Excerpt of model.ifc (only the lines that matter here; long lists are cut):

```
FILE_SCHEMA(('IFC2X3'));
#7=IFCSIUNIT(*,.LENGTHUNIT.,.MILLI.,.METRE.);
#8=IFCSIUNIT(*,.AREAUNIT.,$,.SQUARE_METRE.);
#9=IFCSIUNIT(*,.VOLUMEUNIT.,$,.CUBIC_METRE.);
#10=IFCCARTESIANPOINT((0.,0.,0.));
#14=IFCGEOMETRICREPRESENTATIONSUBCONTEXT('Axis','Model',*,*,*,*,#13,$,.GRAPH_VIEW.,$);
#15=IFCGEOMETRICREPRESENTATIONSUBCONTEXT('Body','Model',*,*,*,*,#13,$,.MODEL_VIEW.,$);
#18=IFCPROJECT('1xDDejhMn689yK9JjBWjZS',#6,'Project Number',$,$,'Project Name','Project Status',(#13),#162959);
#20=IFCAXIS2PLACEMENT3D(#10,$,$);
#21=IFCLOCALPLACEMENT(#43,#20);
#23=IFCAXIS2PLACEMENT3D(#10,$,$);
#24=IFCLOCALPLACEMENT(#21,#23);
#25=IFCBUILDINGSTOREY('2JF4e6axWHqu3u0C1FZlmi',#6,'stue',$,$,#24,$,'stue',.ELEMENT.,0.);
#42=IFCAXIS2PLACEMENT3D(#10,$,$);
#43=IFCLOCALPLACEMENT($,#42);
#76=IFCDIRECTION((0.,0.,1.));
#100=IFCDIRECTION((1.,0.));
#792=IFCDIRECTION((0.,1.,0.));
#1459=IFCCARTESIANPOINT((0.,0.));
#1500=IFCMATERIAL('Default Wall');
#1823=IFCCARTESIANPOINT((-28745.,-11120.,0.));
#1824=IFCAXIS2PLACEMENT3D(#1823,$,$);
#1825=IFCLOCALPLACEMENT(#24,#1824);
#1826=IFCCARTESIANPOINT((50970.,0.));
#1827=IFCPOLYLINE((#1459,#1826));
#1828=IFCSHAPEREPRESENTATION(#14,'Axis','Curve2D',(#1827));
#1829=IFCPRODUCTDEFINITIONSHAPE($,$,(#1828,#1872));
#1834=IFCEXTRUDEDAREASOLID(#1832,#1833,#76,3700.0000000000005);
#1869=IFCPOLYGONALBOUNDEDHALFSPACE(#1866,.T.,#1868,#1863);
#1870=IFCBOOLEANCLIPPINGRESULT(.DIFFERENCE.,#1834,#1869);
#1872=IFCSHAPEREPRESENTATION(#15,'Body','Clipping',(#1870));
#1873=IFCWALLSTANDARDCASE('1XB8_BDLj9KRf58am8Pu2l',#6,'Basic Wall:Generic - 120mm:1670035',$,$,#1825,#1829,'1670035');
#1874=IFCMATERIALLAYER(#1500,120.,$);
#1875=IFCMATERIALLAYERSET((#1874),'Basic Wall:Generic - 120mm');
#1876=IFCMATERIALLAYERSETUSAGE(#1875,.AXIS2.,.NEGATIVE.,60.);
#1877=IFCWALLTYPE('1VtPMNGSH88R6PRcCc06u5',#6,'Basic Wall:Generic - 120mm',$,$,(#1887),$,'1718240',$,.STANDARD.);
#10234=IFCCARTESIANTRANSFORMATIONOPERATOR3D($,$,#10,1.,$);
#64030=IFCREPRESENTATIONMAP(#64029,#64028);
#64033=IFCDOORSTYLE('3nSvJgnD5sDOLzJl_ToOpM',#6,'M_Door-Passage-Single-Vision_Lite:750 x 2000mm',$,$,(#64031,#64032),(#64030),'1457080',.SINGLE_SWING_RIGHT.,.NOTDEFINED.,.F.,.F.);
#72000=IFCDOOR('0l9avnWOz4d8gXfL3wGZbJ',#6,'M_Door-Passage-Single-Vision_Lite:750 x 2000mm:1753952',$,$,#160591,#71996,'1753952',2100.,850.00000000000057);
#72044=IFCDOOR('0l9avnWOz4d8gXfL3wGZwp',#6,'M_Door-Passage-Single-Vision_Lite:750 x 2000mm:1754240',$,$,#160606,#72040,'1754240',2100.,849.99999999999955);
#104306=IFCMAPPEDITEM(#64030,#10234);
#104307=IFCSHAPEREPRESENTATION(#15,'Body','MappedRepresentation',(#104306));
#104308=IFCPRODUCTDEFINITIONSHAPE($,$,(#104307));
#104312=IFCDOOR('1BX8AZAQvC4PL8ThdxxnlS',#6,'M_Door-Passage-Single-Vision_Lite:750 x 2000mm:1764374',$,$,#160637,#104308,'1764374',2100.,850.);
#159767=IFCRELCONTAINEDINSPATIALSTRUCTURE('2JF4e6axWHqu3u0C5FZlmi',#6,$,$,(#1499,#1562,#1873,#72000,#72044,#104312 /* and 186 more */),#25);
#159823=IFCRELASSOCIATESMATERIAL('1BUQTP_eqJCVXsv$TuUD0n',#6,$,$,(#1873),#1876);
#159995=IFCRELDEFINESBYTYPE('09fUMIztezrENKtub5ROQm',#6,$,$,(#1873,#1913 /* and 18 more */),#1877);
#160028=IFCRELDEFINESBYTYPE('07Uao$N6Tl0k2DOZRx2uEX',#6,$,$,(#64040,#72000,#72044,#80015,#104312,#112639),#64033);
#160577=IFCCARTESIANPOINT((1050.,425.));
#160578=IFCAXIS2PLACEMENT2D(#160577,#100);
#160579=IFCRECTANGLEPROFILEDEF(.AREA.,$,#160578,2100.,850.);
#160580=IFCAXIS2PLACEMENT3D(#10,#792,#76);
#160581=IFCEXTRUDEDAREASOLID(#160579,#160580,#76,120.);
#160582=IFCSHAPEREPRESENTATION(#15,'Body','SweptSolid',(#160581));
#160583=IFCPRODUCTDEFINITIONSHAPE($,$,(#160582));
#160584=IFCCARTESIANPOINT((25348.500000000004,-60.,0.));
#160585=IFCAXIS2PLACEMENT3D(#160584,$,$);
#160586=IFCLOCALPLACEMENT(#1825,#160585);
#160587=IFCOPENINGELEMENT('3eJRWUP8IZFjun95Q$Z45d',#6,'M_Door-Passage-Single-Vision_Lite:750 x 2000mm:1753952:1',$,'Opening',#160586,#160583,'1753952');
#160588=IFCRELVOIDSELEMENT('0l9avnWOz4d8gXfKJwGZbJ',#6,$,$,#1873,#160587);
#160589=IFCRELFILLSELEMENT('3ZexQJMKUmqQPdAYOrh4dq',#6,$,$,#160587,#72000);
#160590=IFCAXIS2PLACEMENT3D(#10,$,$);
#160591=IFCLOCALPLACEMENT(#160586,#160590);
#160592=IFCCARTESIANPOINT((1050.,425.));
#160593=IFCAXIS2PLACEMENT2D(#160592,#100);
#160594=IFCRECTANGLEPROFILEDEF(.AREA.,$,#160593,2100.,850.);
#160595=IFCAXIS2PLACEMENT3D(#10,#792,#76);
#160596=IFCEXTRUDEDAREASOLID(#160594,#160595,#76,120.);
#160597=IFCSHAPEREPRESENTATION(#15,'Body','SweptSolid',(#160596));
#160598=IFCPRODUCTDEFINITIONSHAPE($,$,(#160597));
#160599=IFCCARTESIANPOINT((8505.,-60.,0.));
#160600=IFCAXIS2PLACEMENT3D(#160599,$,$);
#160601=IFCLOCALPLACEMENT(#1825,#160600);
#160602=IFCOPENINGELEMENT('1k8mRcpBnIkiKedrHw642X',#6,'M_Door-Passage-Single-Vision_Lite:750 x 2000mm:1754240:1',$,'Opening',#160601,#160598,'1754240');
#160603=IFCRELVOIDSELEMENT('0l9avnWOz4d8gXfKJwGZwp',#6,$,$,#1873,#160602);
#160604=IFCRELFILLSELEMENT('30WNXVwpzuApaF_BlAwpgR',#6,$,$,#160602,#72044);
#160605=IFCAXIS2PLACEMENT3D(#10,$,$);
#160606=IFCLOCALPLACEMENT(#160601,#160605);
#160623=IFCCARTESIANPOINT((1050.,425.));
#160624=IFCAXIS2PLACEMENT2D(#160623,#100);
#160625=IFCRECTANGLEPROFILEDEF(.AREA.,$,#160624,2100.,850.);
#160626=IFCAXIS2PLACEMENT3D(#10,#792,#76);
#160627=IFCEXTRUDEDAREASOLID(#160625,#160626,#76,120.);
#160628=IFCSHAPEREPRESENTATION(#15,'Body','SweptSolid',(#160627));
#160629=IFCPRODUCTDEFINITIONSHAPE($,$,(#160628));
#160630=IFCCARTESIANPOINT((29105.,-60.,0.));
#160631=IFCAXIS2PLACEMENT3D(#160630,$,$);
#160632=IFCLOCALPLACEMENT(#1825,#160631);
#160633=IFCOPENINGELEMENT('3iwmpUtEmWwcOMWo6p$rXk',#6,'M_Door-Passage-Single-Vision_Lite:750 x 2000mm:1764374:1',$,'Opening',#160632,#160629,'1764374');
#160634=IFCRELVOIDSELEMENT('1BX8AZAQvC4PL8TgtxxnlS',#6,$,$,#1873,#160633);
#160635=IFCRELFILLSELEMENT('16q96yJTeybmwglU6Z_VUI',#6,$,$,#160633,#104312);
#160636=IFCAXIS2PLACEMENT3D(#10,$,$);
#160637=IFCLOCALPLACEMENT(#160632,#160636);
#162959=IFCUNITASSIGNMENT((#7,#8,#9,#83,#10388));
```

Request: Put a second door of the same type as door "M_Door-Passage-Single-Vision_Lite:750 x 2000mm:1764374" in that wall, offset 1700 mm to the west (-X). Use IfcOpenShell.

```python
import ifcopenshell
import ifcopenshell.api.feature
import ifcopenshell.api.geometry
import ifcopenshell.api.root
import ifcopenshell.geom
import ifcopenshell.util.element
import ifcopenshell.util.placement
import ifcopenshell.util.shape

model = ifcopenshell.open("model.ifc")
settings = ifcopenshell.geom.settings()


def volume(element):
    """Net volume in cubic metres, openings subtracted."""
    shape = ifcopenshell.geom.create_shape(settings, element)
    return ifcopenshell.util.shape.get_volume(shape.geometry)


def reuse_history(source, copy):
    """copy_class also copies each property set's owner history, people and application; keep the originals."""
    for rel in copy.IsDefinedBy:
        if rel.is_a("IfcRelDefinesByProperties") and (history := rel.RelatingPropertyDefinition.OwnerHistory):
            rel.RelatingPropertyDefinition.OwnerHistory = source.OwnerHistory
            ifcopenshell.util.element.remove_deep2(model, history)


door = model.by_guid("1BX8AZAQvC4PL8ThdxxnlS")
opening = door.FillsVoids[0].RelatingOpeningElement
wall = opening.VoidsElements[0].RelatingBuildingElement
before = volume(wall)
shift = ifcopenshell.util.placement.get_local_placement(wall.ObjectPlacement)[:3, 0] * -1700.0

# copy_class copies the void relationship, type, container and properties, but no geometry.
new_opening = ifcopenshell.api.root.copy_class(model, product=opening)
new_opening.Representation = ifcopenshell.util.element.copy_deep(
    model, opening.Representation, exclude=["IfcGeometricRepresentationContext", "IfcRepresentationMap"]
)
new_opening.Name = "M_Door-Passage-Single-Vision_Lite:750 x 2000mm"
new_opening.Tag = None
new_door = ifcopenshell.api.root.copy_class(model, product=door)
new_door.Representation = ifcopenshell.util.element.copy_deep(
    model, door.Representation, exclude=["IfcGeometricRepresentationContext", "IfcRepresentationMap"]
)
new_door.Name = "M_Door-Passage-Single-Vision_Lite:750 x 2000mm"
new_door.Tag = None
reuse_history(door, new_door)
fills = ifcopenshell.api.feature.add_filling(model, opening=new_opening, element=new_door)
fills.OwnerHistory = new_door.OwnerHistory  # required in IFC2X3

for old, new in ((opening, new_opening), (door, new_door)):
    matrix = ifcopenshell.util.placement.get_local_placement(old.ObjectPlacement)
    matrix[:3, 3] += shift
    ifcopenshell.api.geometry.edit_object_placement(model, product=new, matrix=matrix, is_si=False)

after = volume(wall)

print(f"wall volume {before:.3f} -> {after:.3f} m3")

model.write("model_edited.ifc")
```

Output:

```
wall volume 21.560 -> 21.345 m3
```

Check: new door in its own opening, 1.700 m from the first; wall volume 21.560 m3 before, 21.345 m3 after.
